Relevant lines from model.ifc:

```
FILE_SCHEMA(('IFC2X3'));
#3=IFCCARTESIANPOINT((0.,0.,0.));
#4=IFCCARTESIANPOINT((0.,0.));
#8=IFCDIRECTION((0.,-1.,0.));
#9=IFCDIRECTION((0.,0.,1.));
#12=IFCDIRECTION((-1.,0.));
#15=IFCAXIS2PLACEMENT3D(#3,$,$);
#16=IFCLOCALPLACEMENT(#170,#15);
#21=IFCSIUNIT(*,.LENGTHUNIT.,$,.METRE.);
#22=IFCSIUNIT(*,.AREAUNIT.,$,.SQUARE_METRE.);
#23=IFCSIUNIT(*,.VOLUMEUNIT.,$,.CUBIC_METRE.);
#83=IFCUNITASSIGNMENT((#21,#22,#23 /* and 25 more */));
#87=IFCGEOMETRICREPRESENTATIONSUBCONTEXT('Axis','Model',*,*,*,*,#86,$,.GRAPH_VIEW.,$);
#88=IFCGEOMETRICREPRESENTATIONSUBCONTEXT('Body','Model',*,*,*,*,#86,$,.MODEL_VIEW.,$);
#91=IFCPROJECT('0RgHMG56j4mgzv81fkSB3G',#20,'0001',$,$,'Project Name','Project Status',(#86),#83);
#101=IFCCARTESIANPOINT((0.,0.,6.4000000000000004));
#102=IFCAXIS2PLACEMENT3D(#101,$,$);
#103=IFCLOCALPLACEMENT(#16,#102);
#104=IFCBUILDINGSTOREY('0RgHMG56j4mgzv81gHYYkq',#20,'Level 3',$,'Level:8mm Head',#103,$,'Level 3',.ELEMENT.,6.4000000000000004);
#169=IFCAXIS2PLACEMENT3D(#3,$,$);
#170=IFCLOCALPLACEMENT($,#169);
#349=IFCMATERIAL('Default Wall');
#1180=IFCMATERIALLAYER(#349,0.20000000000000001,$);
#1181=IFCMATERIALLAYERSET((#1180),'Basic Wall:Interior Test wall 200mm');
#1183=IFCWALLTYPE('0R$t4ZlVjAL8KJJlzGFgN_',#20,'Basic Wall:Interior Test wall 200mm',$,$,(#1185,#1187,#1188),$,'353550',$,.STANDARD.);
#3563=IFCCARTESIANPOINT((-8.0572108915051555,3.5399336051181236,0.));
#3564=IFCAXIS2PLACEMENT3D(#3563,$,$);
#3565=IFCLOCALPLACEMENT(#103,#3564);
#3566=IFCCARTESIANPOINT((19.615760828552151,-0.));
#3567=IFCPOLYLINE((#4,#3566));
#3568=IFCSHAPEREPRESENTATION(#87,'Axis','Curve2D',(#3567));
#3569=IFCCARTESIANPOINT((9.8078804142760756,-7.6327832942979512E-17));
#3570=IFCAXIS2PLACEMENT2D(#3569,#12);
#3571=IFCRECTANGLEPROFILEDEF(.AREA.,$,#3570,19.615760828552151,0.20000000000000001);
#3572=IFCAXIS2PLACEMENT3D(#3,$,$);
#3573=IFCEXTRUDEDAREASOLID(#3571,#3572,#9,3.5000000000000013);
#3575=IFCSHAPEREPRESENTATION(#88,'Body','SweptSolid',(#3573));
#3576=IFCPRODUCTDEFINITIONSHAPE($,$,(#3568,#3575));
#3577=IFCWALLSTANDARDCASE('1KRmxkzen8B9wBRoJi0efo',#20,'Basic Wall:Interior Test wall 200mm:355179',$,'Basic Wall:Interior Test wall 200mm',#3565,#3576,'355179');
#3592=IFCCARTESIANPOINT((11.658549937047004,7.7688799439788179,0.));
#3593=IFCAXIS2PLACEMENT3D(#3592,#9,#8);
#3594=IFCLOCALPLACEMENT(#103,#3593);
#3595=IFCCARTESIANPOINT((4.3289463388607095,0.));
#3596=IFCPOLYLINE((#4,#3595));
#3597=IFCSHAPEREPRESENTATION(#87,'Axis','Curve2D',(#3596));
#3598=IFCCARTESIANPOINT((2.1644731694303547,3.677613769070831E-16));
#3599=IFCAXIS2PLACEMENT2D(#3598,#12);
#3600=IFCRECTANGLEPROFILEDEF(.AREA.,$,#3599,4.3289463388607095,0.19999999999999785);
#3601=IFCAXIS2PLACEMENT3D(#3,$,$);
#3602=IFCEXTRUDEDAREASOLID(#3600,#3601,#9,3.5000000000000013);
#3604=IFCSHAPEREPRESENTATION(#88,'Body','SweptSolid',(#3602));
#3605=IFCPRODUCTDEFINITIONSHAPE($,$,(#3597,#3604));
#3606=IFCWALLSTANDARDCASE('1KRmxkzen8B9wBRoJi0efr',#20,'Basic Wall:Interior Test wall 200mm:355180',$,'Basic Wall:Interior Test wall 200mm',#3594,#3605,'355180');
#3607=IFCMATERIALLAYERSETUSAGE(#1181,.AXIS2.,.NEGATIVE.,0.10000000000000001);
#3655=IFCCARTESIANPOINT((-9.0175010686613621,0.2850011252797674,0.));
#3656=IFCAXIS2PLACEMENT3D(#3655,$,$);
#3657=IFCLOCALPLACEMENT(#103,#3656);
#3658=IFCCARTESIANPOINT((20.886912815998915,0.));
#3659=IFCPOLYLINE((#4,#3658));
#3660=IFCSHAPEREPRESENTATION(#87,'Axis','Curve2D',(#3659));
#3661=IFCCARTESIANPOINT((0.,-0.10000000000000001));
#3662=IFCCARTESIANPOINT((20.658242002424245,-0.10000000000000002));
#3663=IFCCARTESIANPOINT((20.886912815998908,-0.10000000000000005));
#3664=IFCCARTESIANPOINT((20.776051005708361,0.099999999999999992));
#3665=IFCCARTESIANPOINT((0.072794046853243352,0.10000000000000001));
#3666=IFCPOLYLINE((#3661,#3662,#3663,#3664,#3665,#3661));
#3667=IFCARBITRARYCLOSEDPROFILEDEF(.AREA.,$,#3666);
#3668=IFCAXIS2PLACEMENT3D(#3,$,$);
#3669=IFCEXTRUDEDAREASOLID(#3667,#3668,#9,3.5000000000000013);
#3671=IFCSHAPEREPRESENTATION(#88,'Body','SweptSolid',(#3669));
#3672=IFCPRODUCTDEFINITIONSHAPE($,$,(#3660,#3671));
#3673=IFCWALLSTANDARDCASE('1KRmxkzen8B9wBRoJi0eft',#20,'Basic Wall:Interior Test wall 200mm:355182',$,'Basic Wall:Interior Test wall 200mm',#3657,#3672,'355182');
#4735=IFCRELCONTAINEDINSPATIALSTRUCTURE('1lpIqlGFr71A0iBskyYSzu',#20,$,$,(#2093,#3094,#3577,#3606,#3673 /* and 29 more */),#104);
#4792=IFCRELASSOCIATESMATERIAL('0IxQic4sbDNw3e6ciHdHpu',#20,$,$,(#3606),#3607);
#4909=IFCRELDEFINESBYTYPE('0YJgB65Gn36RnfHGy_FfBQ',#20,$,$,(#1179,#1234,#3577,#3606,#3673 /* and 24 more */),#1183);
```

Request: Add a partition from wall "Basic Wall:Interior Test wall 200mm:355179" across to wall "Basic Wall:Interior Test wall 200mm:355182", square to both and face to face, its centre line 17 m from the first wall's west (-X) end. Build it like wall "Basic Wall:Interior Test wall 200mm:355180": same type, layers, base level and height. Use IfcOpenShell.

```python
import numpy as np
import ifcopenshell
import ifcopenshell.api.geometry
import ifcopenshell.api.material
import ifcopenshell.api.pset
import ifcopenshell.api.root
import ifcopenshell.api.spatial
import ifcopenshell.api.type
import ifcopenshell.geom
import ifcopenshell.util.element
import ifcopenshell.util.placement
import ifcopenshell.util.representation
import ifcopenshell.util.shape
import ifcopenshell.util.unit

model = ifcopenshell.open("model.ifc")
unit_scale = ifcopenshell.util.unit.calculate_unit_scale(model)
settings = ifcopenshell.geom.settings()
settings.set("use-world-coords", True)

start_wall = model.by_id(3577)
end_wall = model.by_guid("1KRmxkzen8B9wBRoJi0eft")
like = model.by_guid("1KRmxkzen8B9wBRoJi0efr")
matrix = ifcopenshell.util.placement.get_local_placement(start_wall.ObjectPlacement)
matrix[:3, 3] *= unit_scale


def extent(element):
    """Bounding box in the first wall's axes, in metres."""
    shape = ifcopenshell.geom.create_shape(settings, element)
    points = (ifcopenshell.util.shape.get_vertices(shape.geometry) - matrix[:3, 3]) @ matrix[:3, :3]
    return points.min(axis=0), points.max(axis=0)


y_start = extent(start_wall)[0][1]
y_end = extent(end_wall)[1][1]
like_min, like_max = extent(like)
length, height = float(abs(y_end - y_start)), float(like_max[2] - like_min[2])
layer_set = ifcopenshell.util.element.get_material(like, should_skip_usage=True)
thickness = sum(layer.LayerThickness for layer in layer_set.MaterialLayers) * unit_scale

wall = ifcopenshell.api.root.create_entity(model, ifc_class="IfcWallStandardCase", name="New partition")
storey = ifcopenshell.util.element.get_container(like)
ifcopenshell.api.spatial.assign_container(model, products=[wall], relating_structure=storey)
ifcopenshell.api.type.assign_type(
    model, related_objects=[wall], relating_type=ifcopenshell.util.element.get_type(like), should_map_representations=False
)
rel = ifcopenshell.api.material.assign_material(
    model, products=[wall], type="IfcMaterialLayerSetUsage", material=layer_set
)
rel.RelatingMaterial.OffsetFromReferenceLine = -thickness / 2 / unit_scale
pset = ifcopenshell.api.pset.add_pset(model, product=wall, name="Pset_WallCommon")
ifcopenshell.api.pset.edit_pset(model, pset=pset, properties={"IsExternal": False, "LoadBearing": False})

# The axis runs down the middle of the wall.
axis = ifcopenshell.api.geometry.add_axis_representation(
    model, context=ifcopenshell.util.representation.get_context(model, "Model", "Axis"), axis=[(0.0, 0.0), (length, 0.0)]
)
body = ifcopenshell.api.geometry.add_wall_representation(
    model,
    context=ifcopenshell.util.representation.get_context(model, "Model", "Body", "MODEL_VIEW"),
    length=length,
    height=height,
    thickness=thickness,
    offset=-thickness / 2,
)
for representation in (axis, body):
    ifcopenshell.api.geometry.assign_representation(model, product=wall, representation=representation)

placement = matrix @ ifcopenshell.util.placement.rotation(-90, "Z")
placement[:, 3] = matrix @ np.array([extent(start_wall)[0][0] + 17, y_start, like_min[2], 1.0])
ifcopenshell.api.geometry.edit_object_placement(model, product=wall, matrix=placement)

print(f"partition {length:.3f} m long, {height:.3f} m high, {thickness:.3f} m thick")

model.write("model_edited.ifc")
```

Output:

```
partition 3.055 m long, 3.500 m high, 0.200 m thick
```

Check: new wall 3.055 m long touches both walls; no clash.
